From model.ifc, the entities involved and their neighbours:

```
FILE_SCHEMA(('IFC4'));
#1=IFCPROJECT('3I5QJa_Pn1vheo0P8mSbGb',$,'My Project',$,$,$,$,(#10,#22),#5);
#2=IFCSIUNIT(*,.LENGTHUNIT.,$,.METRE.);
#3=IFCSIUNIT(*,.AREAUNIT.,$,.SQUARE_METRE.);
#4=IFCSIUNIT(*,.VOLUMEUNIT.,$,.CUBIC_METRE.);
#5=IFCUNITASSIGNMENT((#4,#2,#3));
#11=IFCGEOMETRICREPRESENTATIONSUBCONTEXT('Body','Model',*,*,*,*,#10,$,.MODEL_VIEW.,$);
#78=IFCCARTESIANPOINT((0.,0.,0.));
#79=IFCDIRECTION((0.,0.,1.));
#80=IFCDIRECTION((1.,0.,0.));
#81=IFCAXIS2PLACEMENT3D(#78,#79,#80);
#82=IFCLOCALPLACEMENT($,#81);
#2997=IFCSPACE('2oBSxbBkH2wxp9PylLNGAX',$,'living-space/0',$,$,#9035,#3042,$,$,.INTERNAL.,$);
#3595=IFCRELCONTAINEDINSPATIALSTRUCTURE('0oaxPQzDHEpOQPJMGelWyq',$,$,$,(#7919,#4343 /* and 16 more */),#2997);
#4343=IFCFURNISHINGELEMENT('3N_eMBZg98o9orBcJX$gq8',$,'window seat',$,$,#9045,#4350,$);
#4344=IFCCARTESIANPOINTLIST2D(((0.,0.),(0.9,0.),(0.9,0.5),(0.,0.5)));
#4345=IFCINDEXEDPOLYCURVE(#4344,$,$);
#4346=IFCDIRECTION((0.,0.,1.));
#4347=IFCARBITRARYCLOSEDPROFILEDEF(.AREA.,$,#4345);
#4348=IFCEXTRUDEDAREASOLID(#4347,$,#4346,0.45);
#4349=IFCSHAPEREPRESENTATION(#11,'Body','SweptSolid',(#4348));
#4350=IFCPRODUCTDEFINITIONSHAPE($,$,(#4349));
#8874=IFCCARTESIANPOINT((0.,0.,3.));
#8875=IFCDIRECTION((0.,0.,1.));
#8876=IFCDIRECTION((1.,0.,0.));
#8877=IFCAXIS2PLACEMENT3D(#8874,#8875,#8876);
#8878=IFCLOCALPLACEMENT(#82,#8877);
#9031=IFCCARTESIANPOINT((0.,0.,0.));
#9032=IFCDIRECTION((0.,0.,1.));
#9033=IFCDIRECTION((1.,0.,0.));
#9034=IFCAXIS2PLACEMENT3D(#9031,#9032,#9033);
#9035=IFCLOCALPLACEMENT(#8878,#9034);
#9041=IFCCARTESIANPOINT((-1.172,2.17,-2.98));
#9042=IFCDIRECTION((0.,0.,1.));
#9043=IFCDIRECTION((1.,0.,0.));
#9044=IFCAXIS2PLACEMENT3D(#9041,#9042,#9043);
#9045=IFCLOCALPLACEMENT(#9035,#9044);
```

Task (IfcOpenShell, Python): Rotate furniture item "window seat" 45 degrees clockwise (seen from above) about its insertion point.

```python
import ifcopenshell
import ifcopenshell.api.geometry
import ifcopenshell.util.placement

model = ifcopenshell.open("model.ifc")

item = model.by_guid("3N_eMBZg98o9orBcJX$gq8")
matrix = ifcopenshell.util.placement.get_local_placement(item.ObjectPlacement)
matrix = matrix @ ifcopenshell.util.placement.rotation(-45, "Z")
ifcopenshell.api.geometry.edit_object_placement(model, product=item, matrix=matrix, is_si=False)

print(ifcopenshell.util.placement.get_local_placement(item.ObjectPlacement).round(3) + 0.0)

model.write("model-out.ifc")
```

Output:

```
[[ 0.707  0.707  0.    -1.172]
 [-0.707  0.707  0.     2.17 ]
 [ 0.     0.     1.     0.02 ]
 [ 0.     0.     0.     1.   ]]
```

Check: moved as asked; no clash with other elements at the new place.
